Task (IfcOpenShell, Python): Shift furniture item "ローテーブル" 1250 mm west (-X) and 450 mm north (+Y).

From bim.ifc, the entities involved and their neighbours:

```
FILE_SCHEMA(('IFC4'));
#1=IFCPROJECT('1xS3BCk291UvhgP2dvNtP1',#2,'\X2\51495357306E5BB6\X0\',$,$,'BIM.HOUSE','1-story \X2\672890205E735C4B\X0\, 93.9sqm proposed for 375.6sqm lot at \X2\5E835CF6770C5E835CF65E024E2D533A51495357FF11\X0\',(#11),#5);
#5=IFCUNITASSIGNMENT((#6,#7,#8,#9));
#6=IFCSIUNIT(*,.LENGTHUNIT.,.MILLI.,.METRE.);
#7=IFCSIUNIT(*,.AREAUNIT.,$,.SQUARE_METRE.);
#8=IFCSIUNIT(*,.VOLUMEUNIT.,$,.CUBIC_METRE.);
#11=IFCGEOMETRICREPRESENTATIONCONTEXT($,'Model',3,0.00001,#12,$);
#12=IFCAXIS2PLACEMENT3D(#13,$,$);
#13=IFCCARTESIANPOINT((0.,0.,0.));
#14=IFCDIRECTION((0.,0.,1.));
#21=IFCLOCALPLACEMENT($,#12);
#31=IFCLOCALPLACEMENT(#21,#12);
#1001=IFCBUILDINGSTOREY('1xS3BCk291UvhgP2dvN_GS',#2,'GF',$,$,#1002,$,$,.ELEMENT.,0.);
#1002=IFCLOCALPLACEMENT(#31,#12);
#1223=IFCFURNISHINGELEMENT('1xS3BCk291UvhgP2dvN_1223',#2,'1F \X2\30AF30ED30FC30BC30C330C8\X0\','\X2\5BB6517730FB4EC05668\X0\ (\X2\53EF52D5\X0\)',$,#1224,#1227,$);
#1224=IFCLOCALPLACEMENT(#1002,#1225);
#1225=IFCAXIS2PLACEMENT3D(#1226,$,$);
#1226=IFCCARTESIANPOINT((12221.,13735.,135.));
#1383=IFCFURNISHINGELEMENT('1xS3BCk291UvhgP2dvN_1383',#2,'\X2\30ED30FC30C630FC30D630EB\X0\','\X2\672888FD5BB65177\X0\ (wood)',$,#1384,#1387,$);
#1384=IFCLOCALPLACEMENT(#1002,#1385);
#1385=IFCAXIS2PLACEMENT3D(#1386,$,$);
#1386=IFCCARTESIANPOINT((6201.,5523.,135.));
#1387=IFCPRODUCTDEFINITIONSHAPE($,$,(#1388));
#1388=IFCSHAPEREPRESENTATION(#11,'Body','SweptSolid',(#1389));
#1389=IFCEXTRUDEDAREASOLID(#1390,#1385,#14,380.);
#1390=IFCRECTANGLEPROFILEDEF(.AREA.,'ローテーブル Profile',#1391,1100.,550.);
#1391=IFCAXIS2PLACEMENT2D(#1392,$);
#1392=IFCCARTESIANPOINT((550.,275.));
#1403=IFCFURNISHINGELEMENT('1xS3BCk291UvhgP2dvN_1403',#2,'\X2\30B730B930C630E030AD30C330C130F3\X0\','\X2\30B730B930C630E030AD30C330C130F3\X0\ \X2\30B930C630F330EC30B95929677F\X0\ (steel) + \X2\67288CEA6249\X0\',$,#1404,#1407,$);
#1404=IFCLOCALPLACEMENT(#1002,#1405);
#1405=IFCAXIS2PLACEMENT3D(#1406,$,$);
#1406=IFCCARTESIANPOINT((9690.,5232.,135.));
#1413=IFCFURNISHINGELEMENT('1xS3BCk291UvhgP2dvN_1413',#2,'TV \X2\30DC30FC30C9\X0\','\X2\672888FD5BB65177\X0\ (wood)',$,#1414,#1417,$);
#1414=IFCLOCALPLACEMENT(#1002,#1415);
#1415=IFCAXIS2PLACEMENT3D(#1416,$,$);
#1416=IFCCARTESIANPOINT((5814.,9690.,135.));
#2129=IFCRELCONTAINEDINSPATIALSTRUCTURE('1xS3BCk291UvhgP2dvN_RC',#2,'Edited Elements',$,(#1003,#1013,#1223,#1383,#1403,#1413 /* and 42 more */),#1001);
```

```python
import ifcopenshell
import ifcopenshell.api.geometry
import ifcopenshell.util.placement

model = ifcopenshell.open("bim.ifc")

item = model.by_guid("1xS3BCk291UvhgP2dvN_1383")
matrix = ifcopenshell.util.placement.get_local_placement(item.ObjectPlacement)
matrix[0, 3] -= 1250.0
matrix[1, 3] += 450.0
ifcopenshell.api.geometry.edit_object_placement(model, product=item, matrix=matrix, is_si=False)

print(ifcopenshell.util.placement.get_local_placement(item.ObjectPlacement).round(3) + 0.0)

model.write("bim-out.ifc")
```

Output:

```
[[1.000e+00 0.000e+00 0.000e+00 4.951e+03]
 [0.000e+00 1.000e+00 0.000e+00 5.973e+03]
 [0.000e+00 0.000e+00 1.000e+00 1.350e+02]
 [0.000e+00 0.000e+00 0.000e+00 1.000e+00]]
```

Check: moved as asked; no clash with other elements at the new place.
